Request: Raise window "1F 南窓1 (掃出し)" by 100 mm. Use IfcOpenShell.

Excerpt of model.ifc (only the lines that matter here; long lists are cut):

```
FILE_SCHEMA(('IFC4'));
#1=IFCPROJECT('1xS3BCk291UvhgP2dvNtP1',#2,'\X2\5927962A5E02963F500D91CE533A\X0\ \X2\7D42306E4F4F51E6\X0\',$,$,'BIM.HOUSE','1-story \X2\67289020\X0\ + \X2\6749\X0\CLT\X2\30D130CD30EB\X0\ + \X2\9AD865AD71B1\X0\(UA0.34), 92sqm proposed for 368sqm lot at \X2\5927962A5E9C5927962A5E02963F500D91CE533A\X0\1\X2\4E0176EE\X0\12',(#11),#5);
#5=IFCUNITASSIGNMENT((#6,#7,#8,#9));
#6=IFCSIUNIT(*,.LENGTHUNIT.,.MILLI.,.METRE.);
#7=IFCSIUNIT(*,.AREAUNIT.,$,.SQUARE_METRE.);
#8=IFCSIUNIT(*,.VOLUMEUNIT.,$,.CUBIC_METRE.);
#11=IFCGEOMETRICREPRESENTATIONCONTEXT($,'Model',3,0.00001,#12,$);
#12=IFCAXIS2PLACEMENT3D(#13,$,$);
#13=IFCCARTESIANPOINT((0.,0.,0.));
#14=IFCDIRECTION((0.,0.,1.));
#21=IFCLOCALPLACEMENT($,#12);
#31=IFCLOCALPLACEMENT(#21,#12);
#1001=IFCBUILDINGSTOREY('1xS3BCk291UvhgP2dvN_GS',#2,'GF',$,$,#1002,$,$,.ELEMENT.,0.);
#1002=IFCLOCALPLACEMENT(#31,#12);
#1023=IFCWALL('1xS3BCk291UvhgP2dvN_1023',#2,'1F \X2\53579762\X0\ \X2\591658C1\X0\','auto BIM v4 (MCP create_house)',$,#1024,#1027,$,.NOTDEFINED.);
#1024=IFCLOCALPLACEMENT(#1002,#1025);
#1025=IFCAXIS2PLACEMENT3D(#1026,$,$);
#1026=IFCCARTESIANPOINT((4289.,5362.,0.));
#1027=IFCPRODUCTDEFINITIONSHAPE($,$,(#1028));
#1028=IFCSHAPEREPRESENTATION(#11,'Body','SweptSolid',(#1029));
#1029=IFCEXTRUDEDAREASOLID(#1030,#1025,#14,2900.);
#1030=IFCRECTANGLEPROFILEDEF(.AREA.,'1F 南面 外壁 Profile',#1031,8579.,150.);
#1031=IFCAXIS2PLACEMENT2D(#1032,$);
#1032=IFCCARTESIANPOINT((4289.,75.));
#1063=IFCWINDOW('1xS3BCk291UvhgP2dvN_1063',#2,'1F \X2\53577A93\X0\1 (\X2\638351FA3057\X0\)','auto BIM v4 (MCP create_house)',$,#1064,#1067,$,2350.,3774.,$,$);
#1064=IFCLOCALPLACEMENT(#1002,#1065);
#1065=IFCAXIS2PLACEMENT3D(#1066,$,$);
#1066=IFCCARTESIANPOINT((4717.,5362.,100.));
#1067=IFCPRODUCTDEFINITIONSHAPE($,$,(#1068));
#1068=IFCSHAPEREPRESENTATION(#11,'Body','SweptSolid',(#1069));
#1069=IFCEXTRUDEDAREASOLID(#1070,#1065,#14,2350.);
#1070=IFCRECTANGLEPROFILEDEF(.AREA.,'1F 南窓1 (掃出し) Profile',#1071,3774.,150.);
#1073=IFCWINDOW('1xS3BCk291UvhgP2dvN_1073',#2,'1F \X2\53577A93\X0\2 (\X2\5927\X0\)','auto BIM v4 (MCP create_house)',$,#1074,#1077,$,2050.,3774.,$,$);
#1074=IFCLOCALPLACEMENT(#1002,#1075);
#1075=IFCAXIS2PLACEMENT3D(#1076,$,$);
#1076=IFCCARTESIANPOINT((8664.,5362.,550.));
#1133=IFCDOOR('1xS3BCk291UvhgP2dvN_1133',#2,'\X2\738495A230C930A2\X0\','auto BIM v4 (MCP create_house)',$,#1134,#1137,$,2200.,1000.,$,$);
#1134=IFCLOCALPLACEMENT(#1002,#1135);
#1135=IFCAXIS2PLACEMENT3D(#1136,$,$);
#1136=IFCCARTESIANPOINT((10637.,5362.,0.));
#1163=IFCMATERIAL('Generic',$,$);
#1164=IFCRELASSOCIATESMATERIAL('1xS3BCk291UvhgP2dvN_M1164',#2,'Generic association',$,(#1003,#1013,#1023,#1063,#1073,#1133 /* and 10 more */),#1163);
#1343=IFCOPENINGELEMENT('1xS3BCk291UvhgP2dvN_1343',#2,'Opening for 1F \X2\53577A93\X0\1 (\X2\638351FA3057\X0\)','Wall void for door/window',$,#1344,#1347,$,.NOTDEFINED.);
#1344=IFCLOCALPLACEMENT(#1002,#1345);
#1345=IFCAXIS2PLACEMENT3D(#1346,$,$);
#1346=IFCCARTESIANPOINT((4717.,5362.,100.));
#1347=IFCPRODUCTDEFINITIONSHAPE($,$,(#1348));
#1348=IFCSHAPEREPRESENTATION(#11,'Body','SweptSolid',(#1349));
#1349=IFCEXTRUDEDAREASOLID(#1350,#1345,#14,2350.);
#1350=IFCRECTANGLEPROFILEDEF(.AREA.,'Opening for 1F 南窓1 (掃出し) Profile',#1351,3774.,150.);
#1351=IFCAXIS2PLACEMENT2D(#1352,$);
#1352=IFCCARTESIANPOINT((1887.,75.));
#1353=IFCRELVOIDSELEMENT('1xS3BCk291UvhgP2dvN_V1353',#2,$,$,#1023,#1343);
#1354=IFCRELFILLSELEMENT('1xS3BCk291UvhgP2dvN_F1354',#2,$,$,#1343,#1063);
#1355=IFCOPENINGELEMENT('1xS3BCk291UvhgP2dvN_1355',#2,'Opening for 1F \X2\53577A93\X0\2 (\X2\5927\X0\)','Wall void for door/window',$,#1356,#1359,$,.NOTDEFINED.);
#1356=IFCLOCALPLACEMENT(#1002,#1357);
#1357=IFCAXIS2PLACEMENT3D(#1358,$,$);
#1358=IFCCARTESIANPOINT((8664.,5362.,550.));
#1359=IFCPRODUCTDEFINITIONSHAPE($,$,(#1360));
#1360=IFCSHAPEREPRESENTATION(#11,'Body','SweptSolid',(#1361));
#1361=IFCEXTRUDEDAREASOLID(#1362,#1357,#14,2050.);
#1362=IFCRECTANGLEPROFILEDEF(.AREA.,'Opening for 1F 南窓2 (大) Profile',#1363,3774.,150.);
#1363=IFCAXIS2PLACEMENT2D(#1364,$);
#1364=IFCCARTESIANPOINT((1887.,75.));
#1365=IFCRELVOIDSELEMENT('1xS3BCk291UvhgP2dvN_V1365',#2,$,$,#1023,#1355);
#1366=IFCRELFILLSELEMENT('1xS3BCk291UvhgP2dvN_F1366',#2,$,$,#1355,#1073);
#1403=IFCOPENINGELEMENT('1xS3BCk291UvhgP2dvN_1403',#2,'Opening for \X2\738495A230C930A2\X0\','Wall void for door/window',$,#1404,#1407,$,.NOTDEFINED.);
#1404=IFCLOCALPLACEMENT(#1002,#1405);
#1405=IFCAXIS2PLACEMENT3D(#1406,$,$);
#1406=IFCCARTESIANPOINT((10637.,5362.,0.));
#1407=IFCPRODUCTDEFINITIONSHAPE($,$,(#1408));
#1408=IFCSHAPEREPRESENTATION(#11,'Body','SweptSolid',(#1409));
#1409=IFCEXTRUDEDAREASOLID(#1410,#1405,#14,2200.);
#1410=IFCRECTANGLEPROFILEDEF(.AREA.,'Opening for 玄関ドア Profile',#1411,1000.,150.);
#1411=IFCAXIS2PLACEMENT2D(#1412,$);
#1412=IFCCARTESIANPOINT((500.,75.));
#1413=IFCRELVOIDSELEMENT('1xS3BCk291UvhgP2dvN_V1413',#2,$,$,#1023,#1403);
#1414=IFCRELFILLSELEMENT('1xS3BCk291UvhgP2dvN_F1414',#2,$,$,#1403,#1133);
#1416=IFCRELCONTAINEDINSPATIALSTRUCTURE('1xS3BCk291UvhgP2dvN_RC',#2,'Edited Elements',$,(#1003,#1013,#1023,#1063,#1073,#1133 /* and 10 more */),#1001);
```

```python
import numpy as np
import ifcopenshell
import ifcopenshell.api.geometry
import ifcopenshell.util.placement
import ifcopenshell.util.unit

model = ifcopenshell.open("model.ifc")
unit_scale = ifcopenshell.util.unit.calculate_unit_scale(model)

window = model.by_id(1063)
opening = window.FillsVoids[0].RelatingOpeningElement
dz = 0.1 / unit_scale

shift = np.array([0.0, 0.0, dz])
# The window is not placed relative to its opening, so move both.
for product in (opening, window):
    matrix = ifcopenshell.util.placement.get_local_placement(product.ObjectPlacement)
    matrix[:3, 3] += shift
    ifcopenshell.api.geometry.edit_object_placement(model, product=product, matrix=matrix, is_si=False)

print(f"moved by {dz * unit_scale:+.3f} m")

model.write("model_v2.ifc")
```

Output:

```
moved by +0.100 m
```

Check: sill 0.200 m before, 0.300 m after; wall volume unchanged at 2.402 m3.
